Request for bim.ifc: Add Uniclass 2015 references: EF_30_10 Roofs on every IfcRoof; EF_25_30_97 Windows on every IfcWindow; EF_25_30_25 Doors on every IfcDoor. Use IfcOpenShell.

First a look at what the model holds.

```python
import ifcopenshell

model = ifcopenshell.open("bim.ifc")
print(model.schema)
print("classifications:", [c.Name for c in model.by_type("IfcClassification")])
for ifc_class in ("IfcDoor", "IfcRoof", "IfcStair", "IfcWall", "IfcWindow"):
    print(ifc_class, len(model.by_type(ifc_class)))
```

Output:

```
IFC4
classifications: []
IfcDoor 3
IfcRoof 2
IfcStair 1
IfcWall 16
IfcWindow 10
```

```python
import ifcopenshell
import ifcopenshell.api.classification

model = ifcopenshell.open("bim.ifc")

system = ifcopenshell.api.classification.add_classification(model, classification="Uniclass 2015")

codes = {
    "IfcRoof": ("EF_30_10", "Roofs"),
    "IfcWindow": ("EF_25_30_97", "Windows"),
    "IfcDoor": ("EF_25_30_25", "Doors"),
}
for ifc_class, (code, name) in codes.items():
    products = model.by_type(ifc_class)
    ifcopenshell.api.classification.add_reference(
        model, products=products, classification=system, identification=code, name=name
    )
    print(code, len(products))

model.write("bim_v2.ifc")
```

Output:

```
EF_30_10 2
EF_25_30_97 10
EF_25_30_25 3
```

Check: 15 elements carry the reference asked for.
